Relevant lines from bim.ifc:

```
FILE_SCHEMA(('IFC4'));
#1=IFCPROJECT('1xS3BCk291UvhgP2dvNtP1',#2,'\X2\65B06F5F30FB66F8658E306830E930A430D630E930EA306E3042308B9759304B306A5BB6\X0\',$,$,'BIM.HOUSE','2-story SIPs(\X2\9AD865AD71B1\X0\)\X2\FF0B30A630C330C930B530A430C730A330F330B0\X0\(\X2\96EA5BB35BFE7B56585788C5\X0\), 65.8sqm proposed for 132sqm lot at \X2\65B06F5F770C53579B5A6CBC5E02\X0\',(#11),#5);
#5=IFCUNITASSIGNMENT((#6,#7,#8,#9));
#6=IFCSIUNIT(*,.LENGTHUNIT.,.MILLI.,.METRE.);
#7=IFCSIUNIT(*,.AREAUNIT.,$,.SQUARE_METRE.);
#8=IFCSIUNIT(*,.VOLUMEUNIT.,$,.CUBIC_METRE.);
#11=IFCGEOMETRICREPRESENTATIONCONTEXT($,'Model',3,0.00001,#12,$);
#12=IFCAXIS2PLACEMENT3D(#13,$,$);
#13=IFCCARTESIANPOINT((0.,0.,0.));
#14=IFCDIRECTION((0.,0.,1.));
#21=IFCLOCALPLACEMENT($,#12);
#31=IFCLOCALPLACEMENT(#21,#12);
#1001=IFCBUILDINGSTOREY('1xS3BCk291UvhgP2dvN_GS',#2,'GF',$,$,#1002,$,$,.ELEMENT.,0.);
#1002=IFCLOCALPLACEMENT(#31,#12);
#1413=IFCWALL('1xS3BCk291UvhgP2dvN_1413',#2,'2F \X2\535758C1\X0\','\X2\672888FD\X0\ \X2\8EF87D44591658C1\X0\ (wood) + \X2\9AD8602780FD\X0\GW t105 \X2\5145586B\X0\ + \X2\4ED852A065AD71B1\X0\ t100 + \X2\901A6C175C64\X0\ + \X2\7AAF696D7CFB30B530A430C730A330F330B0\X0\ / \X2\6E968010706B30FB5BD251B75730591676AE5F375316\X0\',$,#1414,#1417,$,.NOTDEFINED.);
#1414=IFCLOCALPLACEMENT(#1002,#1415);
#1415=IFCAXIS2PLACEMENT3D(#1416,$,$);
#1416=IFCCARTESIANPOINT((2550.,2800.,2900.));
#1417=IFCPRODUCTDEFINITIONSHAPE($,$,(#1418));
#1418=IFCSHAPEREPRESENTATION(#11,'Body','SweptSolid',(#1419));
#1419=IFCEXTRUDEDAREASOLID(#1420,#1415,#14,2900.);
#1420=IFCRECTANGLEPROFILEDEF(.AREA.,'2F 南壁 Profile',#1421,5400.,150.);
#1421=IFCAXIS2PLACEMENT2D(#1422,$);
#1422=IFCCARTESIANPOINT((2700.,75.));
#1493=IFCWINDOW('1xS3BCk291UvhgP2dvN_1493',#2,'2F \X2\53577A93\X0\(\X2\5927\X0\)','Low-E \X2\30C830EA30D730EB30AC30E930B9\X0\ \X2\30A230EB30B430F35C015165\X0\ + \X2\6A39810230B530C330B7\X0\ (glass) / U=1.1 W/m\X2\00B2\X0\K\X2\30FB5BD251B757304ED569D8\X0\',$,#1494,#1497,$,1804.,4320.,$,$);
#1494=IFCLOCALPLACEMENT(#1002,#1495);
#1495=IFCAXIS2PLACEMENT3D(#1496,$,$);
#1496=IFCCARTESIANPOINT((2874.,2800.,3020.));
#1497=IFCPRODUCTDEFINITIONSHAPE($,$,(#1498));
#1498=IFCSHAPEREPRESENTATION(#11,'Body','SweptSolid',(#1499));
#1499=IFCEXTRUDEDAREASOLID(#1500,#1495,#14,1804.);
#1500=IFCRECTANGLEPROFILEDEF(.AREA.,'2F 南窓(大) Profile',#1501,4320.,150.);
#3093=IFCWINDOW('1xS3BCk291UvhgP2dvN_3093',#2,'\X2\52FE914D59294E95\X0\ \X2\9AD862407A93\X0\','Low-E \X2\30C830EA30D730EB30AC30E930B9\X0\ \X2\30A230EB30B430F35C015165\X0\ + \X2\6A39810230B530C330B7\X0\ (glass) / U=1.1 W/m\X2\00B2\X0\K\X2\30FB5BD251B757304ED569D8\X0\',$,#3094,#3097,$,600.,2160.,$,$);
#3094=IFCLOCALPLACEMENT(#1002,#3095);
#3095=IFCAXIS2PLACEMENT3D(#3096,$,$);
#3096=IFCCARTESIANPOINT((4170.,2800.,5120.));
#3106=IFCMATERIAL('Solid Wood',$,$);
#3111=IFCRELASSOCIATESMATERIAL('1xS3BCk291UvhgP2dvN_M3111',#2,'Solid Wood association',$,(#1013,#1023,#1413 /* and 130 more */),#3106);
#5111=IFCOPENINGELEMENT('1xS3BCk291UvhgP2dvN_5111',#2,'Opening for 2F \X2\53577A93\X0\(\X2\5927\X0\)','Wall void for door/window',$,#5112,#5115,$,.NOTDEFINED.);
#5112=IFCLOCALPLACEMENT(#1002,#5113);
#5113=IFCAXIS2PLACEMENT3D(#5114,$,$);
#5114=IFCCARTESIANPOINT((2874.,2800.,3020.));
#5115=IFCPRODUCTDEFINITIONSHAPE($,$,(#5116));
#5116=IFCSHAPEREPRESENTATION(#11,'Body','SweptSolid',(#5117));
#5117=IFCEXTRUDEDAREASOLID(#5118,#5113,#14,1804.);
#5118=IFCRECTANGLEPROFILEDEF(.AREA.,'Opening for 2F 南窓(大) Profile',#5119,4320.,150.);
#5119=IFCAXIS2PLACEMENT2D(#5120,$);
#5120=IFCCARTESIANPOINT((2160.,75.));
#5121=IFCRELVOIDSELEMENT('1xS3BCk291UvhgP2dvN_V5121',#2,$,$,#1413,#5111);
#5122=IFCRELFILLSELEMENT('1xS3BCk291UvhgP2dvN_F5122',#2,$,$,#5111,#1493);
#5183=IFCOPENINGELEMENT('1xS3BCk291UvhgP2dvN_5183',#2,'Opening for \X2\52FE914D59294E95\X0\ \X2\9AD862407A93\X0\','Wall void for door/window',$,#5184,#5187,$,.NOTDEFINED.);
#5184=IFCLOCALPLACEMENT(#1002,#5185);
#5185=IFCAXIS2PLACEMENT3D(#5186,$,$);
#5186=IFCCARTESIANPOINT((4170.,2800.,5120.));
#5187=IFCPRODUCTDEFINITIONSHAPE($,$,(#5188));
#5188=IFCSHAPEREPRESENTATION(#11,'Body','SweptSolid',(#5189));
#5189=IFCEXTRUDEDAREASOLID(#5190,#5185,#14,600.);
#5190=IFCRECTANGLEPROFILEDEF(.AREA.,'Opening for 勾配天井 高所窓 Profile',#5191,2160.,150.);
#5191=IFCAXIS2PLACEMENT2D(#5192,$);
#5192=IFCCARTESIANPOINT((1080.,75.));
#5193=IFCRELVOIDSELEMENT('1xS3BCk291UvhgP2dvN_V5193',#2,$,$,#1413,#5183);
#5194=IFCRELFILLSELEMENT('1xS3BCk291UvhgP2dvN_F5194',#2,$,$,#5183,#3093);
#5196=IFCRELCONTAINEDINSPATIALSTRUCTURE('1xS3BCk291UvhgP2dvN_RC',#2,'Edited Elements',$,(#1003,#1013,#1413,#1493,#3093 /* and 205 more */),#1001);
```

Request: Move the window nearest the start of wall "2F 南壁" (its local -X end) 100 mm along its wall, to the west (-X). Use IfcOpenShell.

```python
import ifcopenshell
import ifcopenshell.api.geometry
import ifcopenshell.util.placement

model = ifcopenshell.open("bim.ifc")

window = model.by_guid("1xS3BCk291UvhgP2dvN_1493")
opening = window.FillsVoids[0].RelatingOpeningElement
wall = opening.VoidsElements[0].RelatingBuildingElement

wall_matrix = ifcopenshell.util.placement.get_local_placement(wall.ObjectPlacement)
shift = wall_matrix[:3, 0] * -100.0
before = ifcopenshell.util.placement.get_local_placement(window.ObjectPlacement)[:3, 3].copy()

# The window is not placed relative to its opening, so move both.
for product in (opening, window):
    matrix = ifcopenshell.util.placement.get_local_placement(product.ObjectPlacement)
    matrix[:3, 3] += shift
    ifcopenshell.api.geometry.edit_object_placement(model, product=product, matrix=matrix, is_si=False)

after = ifcopenshell.util.placement.get_local_placement(window.ObjectPlacement)[:3, 3]
print("window moved by", (after - before).round(3) + 0.0)

model.write("bim_rev.ifc")
```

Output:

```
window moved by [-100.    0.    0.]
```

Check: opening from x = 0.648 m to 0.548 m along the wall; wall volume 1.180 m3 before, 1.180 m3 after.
